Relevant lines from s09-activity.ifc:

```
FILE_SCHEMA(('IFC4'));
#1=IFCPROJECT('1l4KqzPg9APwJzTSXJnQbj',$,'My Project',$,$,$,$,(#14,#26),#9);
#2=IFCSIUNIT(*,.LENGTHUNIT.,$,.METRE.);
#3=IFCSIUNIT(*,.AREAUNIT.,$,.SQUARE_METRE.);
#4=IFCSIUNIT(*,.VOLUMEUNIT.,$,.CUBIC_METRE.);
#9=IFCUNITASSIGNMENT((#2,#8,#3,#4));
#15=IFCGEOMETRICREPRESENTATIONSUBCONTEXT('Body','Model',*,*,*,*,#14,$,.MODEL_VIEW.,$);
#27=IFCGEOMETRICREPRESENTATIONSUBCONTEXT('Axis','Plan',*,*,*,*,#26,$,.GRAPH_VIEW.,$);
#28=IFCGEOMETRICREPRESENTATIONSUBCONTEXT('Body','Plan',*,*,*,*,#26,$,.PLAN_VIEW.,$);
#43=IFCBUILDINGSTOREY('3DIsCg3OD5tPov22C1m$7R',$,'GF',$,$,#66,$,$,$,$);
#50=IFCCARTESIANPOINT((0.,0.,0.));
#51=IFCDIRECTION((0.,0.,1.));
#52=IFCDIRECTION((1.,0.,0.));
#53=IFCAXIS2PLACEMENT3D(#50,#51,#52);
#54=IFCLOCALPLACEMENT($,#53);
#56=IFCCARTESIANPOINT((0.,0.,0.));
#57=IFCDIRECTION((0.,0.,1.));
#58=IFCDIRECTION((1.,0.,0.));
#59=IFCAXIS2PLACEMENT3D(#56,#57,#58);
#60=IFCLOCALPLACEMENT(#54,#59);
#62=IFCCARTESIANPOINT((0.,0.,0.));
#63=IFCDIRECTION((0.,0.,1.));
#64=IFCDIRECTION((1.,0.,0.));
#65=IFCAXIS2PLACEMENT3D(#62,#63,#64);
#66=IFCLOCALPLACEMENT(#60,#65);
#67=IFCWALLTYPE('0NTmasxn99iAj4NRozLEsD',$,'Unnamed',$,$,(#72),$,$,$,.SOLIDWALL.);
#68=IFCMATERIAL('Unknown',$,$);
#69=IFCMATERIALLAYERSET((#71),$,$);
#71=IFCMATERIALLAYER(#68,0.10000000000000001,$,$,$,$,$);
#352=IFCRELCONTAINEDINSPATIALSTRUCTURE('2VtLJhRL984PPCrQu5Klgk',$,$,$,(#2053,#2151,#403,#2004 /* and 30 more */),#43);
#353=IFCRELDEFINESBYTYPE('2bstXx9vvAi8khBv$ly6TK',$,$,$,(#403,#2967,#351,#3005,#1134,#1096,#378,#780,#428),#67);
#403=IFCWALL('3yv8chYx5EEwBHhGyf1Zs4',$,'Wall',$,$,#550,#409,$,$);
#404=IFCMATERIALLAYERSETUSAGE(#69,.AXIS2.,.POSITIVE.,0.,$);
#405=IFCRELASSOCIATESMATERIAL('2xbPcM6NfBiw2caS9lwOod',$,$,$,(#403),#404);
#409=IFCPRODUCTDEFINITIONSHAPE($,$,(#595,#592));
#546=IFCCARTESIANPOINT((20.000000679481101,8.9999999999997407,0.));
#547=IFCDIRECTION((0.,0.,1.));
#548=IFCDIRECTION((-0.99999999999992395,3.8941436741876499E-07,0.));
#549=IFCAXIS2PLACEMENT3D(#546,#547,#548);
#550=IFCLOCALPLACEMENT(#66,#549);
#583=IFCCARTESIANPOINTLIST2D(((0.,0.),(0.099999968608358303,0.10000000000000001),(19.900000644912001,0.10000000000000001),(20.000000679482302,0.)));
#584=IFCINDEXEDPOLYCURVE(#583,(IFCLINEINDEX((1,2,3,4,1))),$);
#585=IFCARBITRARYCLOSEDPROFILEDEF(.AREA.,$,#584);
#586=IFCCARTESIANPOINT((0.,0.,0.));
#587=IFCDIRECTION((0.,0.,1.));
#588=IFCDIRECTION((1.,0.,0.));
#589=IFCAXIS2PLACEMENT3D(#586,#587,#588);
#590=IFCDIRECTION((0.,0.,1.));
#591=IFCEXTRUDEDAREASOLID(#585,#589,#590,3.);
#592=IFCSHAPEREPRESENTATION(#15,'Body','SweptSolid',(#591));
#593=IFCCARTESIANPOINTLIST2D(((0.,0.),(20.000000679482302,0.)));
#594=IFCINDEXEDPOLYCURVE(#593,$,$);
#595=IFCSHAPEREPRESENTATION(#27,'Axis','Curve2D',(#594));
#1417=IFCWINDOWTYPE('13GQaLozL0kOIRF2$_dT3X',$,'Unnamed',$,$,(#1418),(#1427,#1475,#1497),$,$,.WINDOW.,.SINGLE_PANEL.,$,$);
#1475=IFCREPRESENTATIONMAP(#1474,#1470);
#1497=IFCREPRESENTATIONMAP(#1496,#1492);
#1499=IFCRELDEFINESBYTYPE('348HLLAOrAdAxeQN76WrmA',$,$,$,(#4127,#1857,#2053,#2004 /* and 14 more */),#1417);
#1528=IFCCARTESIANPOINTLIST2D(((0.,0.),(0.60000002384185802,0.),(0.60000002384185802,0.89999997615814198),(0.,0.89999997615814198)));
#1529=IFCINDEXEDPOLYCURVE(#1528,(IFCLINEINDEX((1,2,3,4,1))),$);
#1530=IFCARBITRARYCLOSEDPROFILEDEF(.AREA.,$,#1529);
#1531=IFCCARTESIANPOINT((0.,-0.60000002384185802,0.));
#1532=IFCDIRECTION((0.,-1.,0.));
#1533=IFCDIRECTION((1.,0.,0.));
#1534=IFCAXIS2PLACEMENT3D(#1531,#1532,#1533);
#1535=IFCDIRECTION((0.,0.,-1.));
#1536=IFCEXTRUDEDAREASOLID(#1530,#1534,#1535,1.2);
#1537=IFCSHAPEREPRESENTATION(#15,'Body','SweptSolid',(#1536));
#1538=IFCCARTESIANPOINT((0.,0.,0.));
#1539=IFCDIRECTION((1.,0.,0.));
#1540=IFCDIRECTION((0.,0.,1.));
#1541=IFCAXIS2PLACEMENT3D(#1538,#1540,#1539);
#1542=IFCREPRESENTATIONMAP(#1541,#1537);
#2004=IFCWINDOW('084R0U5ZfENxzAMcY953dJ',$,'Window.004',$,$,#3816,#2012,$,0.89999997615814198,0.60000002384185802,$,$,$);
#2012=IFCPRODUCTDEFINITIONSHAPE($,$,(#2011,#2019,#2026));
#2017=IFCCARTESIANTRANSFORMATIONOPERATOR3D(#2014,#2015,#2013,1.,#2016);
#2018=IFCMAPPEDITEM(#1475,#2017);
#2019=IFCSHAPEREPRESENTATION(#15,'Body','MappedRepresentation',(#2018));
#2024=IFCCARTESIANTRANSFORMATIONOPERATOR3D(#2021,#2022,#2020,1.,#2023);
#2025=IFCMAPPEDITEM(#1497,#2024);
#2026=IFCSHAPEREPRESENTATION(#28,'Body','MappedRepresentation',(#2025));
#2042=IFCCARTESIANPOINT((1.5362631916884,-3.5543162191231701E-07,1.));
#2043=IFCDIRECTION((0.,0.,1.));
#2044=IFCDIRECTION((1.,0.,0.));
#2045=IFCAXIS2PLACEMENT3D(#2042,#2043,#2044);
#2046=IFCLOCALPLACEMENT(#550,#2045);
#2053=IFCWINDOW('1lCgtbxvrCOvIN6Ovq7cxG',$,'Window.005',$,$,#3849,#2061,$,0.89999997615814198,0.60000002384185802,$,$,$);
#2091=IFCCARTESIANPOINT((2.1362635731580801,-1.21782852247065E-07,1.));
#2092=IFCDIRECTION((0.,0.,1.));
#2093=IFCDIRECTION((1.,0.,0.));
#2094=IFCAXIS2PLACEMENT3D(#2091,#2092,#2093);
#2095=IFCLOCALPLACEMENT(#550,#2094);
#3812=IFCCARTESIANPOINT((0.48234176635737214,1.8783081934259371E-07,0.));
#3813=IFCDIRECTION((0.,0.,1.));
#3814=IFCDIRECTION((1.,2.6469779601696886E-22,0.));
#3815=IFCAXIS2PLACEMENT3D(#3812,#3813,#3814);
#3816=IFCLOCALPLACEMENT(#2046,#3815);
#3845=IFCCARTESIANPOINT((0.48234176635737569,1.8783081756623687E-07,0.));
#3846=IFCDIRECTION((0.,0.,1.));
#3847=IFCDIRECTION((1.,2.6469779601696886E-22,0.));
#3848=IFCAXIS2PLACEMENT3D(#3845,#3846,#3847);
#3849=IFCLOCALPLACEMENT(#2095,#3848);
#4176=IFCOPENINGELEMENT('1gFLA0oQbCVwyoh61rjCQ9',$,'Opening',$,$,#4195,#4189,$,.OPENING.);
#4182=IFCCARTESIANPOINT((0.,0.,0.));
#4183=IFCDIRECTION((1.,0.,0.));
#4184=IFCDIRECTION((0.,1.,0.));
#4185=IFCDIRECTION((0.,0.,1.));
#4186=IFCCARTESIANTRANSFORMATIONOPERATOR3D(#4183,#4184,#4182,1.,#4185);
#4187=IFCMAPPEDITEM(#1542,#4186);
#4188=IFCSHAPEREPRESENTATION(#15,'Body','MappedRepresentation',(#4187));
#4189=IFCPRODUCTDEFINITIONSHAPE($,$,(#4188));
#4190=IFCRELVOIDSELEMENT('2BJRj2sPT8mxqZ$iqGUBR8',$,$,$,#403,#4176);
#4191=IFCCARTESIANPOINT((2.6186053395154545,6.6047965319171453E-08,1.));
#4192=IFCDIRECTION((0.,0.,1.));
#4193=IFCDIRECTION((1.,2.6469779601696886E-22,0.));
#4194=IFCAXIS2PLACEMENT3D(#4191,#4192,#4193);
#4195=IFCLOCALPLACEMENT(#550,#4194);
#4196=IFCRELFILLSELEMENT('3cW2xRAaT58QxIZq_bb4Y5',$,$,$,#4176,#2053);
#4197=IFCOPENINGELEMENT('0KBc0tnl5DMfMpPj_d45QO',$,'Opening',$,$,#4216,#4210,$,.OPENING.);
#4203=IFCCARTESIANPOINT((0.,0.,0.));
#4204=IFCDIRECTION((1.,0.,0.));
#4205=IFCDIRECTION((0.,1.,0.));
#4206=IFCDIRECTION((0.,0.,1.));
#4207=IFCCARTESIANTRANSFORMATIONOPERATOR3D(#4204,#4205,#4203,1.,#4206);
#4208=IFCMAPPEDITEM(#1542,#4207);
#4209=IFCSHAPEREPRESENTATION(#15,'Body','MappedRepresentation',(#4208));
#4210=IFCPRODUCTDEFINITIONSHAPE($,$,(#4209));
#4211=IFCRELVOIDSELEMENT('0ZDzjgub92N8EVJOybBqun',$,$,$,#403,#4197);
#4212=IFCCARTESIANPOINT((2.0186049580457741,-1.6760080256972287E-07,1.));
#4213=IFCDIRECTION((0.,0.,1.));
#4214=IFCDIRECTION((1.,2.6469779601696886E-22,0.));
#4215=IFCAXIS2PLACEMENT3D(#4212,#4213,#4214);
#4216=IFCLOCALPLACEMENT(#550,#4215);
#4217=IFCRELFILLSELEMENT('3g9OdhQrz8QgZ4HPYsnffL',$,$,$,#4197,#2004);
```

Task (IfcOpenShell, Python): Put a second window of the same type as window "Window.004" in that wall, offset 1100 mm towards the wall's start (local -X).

```python
import ifcopenshell
import ifcopenshell.api.feature
import ifcopenshell.api.geometry
import ifcopenshell.api.root
import ifcopenshell.geom
import ifcopenshell.util.element
import ifcopenshell.util.placement
import ifcopenshell.util.shape

model = ifcopenshell.open("s09-activity.ifc")
settings = ifcopenshell.geom.settings()


def volume(element):
    """Net volume in cubic metres, openings subtracted."""
    shape = ifcopenshell.geom.create_shape(settings, element)
    return ifcopenshell.util.shape.get_volume(shape.geometry)


window = model.by_id(2004)
opening = window.FillsVoids[0].RelatingOpeningElement
wall = opening.VoidsElements[0].RelatingBuildingElement
before = volume(wall)
shift = ifcopenshell.util.placement.get_local_placement(wall.ObjectPlacement)[:3, 0] * -1.1

# copy_class copies the void relationship, type, container and properties, but no geometry.
new_opening = ifcopenshell.api.root.copy_class(model, product=opening)
new_opening.Representation = ifcopenshell.util.element.copy_deep(
    model, opening.Representation, exclude=["IfcGeometricRepresentationContext", "IfcRepresentationMap"]
)
new_window = ifcopenshell.api.root.copy_class(model, product=window)
new_window.Representation = ifcopenshell.util.element.copy_deep(
    model, window.Representation, exclude=["IfcGeometricRepresentationContext", "IfcRepresentationMap"]
)
ifcopenshell.api.feature.add_filling(model, opening=new_opening, element=new_window)

for old, new in ((opening, new_opening), (window, new_window)):
    matrix = ifcopenshell.util.placement.get_local_placement(old.ObjectPlacement)
    matrix[:3, 3] += shift
    ifcopenshell.api.geometry.edit_object_placement(model, product=new, matrix=matrix, is_si=False)

after = volume(wall)

print(f"wall volume {before:.3f} -> {after:.3f} m3")

model.write("s09-activity-out.ifc")
```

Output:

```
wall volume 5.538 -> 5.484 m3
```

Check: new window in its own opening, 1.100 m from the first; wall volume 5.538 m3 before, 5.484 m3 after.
